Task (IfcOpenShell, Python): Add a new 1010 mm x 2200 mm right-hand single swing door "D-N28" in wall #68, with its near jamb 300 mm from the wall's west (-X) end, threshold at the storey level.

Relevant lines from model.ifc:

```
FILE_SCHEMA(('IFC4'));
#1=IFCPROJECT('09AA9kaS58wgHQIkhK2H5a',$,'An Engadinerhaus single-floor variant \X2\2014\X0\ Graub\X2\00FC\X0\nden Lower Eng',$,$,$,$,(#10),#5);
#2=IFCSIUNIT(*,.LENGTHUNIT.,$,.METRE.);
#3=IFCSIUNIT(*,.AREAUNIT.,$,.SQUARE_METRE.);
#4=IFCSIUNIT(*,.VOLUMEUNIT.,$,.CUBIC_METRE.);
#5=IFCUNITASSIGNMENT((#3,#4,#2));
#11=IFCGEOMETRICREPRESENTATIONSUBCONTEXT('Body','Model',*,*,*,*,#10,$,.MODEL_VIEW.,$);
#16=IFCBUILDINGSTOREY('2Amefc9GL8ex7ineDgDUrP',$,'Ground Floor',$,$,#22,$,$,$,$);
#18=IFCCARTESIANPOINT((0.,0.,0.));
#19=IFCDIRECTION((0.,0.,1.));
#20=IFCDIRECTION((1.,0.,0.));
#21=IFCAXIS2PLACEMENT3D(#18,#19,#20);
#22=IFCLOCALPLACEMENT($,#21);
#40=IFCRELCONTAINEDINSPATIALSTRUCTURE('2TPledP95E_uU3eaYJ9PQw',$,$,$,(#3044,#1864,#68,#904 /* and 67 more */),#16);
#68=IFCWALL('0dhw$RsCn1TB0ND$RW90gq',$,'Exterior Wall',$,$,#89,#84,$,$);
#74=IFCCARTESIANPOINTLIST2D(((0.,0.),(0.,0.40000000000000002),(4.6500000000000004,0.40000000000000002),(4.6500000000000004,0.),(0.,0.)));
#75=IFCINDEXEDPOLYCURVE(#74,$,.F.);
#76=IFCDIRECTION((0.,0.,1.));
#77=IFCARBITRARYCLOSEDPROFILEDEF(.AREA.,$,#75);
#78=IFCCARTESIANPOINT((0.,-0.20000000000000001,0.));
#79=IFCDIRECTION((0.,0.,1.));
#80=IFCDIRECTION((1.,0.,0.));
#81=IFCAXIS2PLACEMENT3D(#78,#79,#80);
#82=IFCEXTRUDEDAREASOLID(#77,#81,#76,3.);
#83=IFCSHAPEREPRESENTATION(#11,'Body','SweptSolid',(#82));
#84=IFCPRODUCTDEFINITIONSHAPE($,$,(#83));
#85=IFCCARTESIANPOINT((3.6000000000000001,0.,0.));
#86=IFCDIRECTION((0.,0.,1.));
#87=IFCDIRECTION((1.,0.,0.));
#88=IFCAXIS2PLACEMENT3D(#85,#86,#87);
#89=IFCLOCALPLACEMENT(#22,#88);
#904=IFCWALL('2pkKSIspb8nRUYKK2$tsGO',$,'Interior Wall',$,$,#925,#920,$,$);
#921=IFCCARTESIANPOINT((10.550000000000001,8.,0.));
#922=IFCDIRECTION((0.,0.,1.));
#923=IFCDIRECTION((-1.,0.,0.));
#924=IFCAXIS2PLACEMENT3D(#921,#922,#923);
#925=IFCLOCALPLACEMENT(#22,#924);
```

```python
import numpy as np
import ifcopenshell
import ifcopenshell.api.feature
import ifcopenshell.api.geometry
import ifcopenshell.api.root
import ifcopenshell.api.spatial
import ifcopenshell.geom
import ifcopenshell.util.element
import ifcopenshell.util.placement
import ifcopenshell.util.representation
import ifcopenshell.util.shape
import ifcopenshell.util.unit

model = ifcopenshell.open("model.ifc")
unit_scale = ifcopenshell.util.unit.calculate_unit_scale(model)
settings = ifcopenshell.geom.settings()


def volume(element):
    """Net volume in cubic metres, openings subtracted."""
    shape = ifcopenshell.geom.create_shape(settings, element)
    return ifcopenshell.util.shape.get_volume(shape.geometry)


wall = model.by_guid("0dhw$RsCn1TB0ND$RW90gq")
storey = ifcopenshell.util.element.get_container(wall, ifc_class="IfcBuildingStorey")
context = ifcopenshell.util.representation.get_context(model, "Model", "Body", "MODEL_VIEW")
before = volume(wall)

width, height, from_end, sill = 1.01, 2.2, 0.3, 0.0  # metres

# The wall runs along its own X axis, and the end named is its -X end.
wall_shape = ifcopenshell.geom.create_shape(settings, wall)
x, y, z = ifcopenshell.util.shape.get_vertices(wall_shape.geometry).T
start = x.min() + from_end
face, thickness = float(y.min()), float(y.max() - y.min())
wall_matrix = ifcopenshell.util.placement.get_local_placement(wall.ObjectPlacement)
level = ifcopenshell.util.placement.get_local_placement(storey.ObjectPlacement)[2, 3]


def in_wall(x, y):
    """Placement at x, y metres in the wall's axes, at sill height."""
    matrix = wall_matrix.copy()
    matrix[:, 3] = wall_matrix @ np.array([x / unit_scale, y / unit_scale, 0.0, 1.0])
    matrix[2, 3] = level + sill / unit_scale
    return matrix


# Opening: a box that overshoots both wall faces by 50 mm.
opening = ifcopenshell.api.root.create_entity(model, ifc_class="IfcOpeningElement", predefined_type="OPENING")
box = ifcopenshell.api.geometry.add_wall_representation(
    model, context=context, length=width, height=height, thickness=thickness + 0.1
)
ifcopenshell.api.geometry.assign_representation(model, product=opening, representation=box)
ifcopenshell.api.geometry.edit_object_placement(model, product=opening, matrix=in_wall(start, face - 0.05), is_si=False)
ifcopenshell.api.feature.add_feature(model, feature=opening, element=wall)

door = ifcopenshell.api.root.create_entity(model, ifc_class="IfcDoor", name="D-N28", predefined_type="DOOR")
door.OverallWidth, door.OverallHeight = width / unit_scale, height / unit_scale
door.OperationType = "SINGLE_SWING_RIGHT"
body = ifcopenshell.api.geometry.add_door_representation(
    model,
    context=context,
    overall_width=door.OverallWidth,
    overall_height=door.OverallHeight,
    operation_type="SINGLE_SWING_RIGHT",
    lining_properties={"LiningDepth": thickness / unit_scale, "ThresholdDepth": thickness / unit_scale},
)
ifcopenshell.api.geometry.assign_representation(model, product=door, representation=body)
ifcopenshell.api.spatial.assign_container(model, products=[door], relating_structure=storey)
ifcopenshell.api.feature.add_filling(model, opening=opening, element=door)

# The lining spans the wall, so the door starts at the wall face.
ifcopenshell.api.geometry.edit_object_placement(model, product=door, matrix=in_wall(start, face), is_si=False)

after = volume(wall)

print(f"wall volume {before:.3f} -> {after:.3f} m3")

model.write("model-out.ifc")
```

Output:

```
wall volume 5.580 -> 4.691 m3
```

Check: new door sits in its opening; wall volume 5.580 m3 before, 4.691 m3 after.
